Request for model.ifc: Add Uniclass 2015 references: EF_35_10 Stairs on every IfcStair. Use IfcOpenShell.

First a look at what the model holds.

```python
import ifcopenshell

model = ifcopenshell.open("model.ifc")
print(model.schema)
print("classifications:", [c.Name for c in model.by_type("IfcClassification")])
for ifc_class in ("IfcDoor", "IfcRoof", "IfcStair", "IfcWall", "IfcWindow"):
    print(ifc_class, len(model.by_type(ifc_class)))
```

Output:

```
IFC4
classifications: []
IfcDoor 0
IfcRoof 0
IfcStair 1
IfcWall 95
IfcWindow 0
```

```python
import ifcopenshell
import ifcopenshell.api.classification

model = ifcopenshell.open("model.ifc")

system = ifcopenshell.api.classification.add_classification(model, classification="Uniclass 2015")

codes = {
    "IfcStair": ("EF_35_10", "Stairs"),
}
for ifc_class, (code, name) in codes.items():
    products = model.by_type(ifc_class)
    ifcopenshell.api.classification.add_reference(
        model, products=products, classification=system, identification=code, name=name
    )
    print(code, len(products))

model.write("model-out.ifc")
```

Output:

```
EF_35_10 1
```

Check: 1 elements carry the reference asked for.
